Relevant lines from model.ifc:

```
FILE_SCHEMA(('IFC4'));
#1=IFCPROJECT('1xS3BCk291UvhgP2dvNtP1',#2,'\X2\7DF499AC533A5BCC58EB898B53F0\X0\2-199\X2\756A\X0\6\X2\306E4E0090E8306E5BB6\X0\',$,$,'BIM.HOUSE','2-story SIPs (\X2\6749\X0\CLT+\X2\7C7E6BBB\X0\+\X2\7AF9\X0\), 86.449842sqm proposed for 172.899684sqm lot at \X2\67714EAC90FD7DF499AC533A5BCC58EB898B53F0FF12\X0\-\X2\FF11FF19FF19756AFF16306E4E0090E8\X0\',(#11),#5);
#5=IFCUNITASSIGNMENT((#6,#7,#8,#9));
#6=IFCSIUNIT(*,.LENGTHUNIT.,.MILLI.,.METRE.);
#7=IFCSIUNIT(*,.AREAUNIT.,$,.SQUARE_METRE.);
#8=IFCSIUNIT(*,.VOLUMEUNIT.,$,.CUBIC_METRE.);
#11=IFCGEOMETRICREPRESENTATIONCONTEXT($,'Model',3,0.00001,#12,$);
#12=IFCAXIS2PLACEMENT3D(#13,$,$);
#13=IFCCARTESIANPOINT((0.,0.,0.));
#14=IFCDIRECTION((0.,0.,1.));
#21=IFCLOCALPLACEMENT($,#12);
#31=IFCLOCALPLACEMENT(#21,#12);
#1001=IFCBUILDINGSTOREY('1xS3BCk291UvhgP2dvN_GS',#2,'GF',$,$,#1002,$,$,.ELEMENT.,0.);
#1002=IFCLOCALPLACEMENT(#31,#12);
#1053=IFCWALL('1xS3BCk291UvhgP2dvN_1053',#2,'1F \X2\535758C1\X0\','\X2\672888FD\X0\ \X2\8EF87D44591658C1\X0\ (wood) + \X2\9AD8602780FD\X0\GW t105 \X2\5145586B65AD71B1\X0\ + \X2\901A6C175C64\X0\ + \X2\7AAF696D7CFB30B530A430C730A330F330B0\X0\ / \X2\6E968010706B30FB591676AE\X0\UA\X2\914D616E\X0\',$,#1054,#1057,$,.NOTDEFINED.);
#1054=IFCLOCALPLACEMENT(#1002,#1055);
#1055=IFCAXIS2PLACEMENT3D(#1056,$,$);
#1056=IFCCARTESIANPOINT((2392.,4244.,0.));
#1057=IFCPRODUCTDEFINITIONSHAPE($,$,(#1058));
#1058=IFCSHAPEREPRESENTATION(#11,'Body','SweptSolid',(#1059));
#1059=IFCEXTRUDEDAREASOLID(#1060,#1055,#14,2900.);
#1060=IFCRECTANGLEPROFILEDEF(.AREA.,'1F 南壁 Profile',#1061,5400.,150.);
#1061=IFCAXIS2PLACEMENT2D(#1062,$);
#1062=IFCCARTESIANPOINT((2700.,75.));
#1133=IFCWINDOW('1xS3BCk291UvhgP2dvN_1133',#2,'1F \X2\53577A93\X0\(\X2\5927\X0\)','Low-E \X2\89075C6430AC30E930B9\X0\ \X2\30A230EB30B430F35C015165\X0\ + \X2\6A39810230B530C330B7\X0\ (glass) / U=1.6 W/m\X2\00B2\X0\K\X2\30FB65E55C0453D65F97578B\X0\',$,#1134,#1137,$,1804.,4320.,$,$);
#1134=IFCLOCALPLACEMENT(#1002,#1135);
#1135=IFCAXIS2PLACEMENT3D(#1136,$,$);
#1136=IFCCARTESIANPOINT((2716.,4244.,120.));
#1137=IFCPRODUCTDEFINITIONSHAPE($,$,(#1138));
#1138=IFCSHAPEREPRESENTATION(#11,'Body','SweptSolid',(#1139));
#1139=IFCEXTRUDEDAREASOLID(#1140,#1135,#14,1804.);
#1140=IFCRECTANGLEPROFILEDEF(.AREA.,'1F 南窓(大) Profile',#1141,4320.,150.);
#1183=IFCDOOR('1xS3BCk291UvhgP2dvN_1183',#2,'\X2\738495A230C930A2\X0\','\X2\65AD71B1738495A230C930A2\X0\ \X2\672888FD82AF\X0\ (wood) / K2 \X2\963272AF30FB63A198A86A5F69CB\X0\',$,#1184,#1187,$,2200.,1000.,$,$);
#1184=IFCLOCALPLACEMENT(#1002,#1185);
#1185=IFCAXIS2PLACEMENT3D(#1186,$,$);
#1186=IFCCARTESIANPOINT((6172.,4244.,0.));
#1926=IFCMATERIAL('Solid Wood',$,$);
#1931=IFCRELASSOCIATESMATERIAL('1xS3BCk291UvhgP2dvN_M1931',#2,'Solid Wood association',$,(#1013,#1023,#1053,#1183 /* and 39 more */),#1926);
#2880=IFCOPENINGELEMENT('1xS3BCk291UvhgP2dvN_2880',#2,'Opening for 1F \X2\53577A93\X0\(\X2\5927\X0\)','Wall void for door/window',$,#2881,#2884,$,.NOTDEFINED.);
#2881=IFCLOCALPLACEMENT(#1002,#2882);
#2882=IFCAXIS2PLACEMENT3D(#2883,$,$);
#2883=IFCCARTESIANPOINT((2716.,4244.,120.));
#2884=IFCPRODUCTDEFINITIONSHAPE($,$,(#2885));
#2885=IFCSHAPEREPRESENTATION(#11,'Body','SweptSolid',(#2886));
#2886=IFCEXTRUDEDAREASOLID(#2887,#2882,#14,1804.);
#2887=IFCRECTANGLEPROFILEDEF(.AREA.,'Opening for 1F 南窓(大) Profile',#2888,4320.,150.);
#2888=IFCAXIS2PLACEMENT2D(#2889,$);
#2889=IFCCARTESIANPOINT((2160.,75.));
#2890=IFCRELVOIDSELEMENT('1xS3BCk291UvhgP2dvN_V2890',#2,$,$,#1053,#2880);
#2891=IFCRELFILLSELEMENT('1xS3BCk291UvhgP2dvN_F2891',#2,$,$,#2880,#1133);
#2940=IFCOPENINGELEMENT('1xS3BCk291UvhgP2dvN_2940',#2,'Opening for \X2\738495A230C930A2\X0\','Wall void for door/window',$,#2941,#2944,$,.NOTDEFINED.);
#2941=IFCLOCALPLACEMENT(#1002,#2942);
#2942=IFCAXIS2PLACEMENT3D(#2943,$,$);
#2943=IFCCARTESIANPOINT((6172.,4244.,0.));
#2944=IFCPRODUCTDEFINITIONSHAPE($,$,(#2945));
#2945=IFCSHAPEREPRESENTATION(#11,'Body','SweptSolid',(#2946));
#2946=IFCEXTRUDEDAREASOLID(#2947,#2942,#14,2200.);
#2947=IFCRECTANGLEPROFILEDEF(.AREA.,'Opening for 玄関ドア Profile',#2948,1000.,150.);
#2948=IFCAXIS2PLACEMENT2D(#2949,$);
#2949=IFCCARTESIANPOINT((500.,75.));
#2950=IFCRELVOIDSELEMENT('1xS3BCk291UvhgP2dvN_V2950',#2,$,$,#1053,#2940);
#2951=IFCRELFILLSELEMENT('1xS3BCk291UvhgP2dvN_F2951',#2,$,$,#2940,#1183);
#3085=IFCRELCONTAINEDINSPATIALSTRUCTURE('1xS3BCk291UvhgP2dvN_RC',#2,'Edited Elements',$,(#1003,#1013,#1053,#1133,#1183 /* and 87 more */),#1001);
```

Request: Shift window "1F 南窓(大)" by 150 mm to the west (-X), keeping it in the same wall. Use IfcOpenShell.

```python
import ifcopenshell
import ifcopenshell.api.geometry
import ifcopenshell.util.placement
import ifcopenshell.util.unit

model = ifcopenshell.open("model.ifc")
unit_scale = ifcopenshell.util.unit.calculate_unit_scale(model)

window = model.by_id(1133)
opening = window.FillsVoids[0].RelatingOpeningElement
wall = opening.VoidsElements[0].RelatingBuildingElement

wall_matrix = ifcopenshell.util.placement.get_local_placement(wall.ObjectPlacement)
shift = wall_matrix[:3, 0] * -0.15 / unit_scale
before = ifcopenshell.util.placement.get_local_placement(window.ObjectPlacement)[:3, 3].copy()

# The window is not placed relative to its opening, so move both.
for product in (opening, window):
    matrix = ifcopenshell.util.placement.get_local_placement(product.ObjectPlacement)
    matrix[:3, 3] += shift
    ifcopenshell.api.geometry.edit_object_placement(model, product=product, matrix=matrix, is_si=False)

after = ifcopenshell.util.placement.get_local_placement(window.ObjectPlacement)[:3, 3]
print("window moved by", (after - before).round(3) + 0.0)

model.write("model_v2.ifc")
```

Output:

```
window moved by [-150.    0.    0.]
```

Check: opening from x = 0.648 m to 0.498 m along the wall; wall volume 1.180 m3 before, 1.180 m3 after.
